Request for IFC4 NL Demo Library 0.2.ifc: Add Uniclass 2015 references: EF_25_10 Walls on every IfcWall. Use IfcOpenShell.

First a look at what the model holds.

```python
import ifcopenshell

model = ifcopenshell.open("IFC4 NL Demo Library 0.2.ifc")
print(model.schema)
print("classifications:", [c.Name for c in model.by_type("IfcClassification")])
for ifc_class in ("IfcDoor", "IfcRoof", "IfcStair", "IfcWall", "IfcWindow"):
    print(ifc_class, len(model.by_type(ifc_class)))
```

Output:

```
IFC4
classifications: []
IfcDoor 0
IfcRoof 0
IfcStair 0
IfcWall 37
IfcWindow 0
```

```python
import ifcopenshell
import ifcopenshell.api.classification

model = ifcopenshell.open("IFC4 NL Demo Library 0.2.ifc")

system = ifcopenshell.api.classification.add_classification(model, classification="Uniclass 2015")

codes = {
    "IfcWall": ("EF_25_10", "Walls"),
}
for ifc_class, (code, name) in codes.items():
    products = model.by_type(ifc_class)
    ifcopenshell.api.classification.add_reference(
        model, products=products, classification=system, identification=code, name=name
    )
    print(code, len(products))

model.write("IFC4 NL Demo Library 0.2_updated.ifc")
```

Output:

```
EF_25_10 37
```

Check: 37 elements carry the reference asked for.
